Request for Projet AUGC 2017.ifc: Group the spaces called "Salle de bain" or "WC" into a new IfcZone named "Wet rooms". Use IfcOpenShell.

First a look at what the model holds.

```python
import ifcopenshell

model = ifcopenshell.open("Projet AUGC 2017.ifc")
print(model.schema)
seen = {}
for space in model.by_type("IfcSpace"):
    seen[space.LongName] = seen.get(space.LongName, 0) + 1
for name, count in sorted(seen.items(), key=str):
    print(count, "x", name)
print("zones:", [z.Name for z in model.by_type("IfcZone")][:20])
```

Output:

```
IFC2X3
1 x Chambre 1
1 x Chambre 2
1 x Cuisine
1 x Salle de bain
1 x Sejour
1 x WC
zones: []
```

```python
import ifcopenshell
import ifcopenshell.api.group
import ifcopenshell.api.root

model = ifcopenshell.open("Projet AUGC 2017.ifc")

names = {"Salle de bain", "WC"}
spaces = [s for s in model.by_type("IfcSpace") if s.LongName in names]

zone = ifcopenshell.api.root.create_entity(model, ifc_class="IfcZone", name="Wet rooms")
ifcopenshell.api.group.assign_group(model, products=spaces, group=zone)
print(len(spaces), "spaces in", zone.Name)

model.write("Projet AUGC 2017-out.ifc")
```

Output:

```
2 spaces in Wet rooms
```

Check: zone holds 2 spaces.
